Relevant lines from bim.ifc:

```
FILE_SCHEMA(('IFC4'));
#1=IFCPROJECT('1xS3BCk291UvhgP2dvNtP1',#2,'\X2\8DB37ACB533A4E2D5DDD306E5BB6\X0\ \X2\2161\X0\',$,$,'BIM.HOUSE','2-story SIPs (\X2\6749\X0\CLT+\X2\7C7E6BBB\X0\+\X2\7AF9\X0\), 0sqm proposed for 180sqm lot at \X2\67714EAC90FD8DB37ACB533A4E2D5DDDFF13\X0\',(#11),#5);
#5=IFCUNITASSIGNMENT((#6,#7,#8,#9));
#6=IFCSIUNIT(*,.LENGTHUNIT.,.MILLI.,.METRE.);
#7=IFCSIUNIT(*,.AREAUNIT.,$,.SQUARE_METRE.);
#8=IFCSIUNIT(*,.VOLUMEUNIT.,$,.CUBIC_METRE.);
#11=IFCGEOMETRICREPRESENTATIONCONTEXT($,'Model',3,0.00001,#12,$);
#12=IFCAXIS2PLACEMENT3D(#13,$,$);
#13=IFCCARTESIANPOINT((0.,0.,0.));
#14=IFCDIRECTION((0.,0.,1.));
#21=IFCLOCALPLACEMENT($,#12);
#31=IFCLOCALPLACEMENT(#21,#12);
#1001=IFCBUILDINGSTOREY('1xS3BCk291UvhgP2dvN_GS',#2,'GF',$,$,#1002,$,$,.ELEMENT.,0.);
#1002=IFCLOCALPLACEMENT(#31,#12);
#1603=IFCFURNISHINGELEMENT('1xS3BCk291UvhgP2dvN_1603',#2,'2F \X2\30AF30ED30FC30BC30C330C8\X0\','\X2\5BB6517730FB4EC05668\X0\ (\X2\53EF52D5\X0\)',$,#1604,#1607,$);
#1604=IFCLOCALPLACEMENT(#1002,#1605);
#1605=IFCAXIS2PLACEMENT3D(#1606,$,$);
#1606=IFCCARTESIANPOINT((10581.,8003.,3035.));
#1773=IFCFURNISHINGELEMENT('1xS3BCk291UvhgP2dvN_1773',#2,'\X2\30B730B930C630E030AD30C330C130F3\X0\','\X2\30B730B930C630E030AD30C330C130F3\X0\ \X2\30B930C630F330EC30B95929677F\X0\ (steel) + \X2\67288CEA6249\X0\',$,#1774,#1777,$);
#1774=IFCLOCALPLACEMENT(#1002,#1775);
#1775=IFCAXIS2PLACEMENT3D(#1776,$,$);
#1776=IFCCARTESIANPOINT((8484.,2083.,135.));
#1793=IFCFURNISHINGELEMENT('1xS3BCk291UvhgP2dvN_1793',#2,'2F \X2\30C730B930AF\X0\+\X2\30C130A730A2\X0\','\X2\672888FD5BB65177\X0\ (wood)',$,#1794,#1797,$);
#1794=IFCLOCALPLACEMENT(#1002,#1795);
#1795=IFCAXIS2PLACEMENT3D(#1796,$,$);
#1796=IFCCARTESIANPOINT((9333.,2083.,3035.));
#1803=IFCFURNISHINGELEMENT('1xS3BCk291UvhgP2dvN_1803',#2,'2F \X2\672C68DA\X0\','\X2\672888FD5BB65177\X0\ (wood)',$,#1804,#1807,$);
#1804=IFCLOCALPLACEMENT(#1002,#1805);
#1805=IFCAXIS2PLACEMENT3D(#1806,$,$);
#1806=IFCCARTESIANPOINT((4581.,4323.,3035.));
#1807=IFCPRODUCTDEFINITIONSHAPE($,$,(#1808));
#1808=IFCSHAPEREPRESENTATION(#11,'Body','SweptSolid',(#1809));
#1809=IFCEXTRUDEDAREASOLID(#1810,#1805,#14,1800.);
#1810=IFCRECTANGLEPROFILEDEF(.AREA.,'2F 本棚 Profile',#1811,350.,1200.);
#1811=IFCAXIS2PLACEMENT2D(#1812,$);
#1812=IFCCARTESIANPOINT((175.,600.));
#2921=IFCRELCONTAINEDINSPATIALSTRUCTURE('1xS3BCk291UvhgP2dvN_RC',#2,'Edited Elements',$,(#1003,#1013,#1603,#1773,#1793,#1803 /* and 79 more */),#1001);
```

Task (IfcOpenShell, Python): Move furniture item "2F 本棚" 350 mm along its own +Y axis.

```python
import ifcopenshell
import ifcopenshell.api.geometry
import ifcopenshell.util.placement

model = ifcopenshell.open("bim.ifc")

item = model.by_id(1803)
matrix = ifcopenshell.util.placement.get_local_placement(item.ObjectPlacement)
matrix[:3, 3] += matrix[:3, 1] * 350.0
ifcopenshell.api.geometry.edit_object_placement(model, product=item, matrix=matrix, is_si=False)

print(ifcopenshell.util.placement.get_local_placement(item.ObjectPlacement).round(3) + 0.0)

model.write("bim_v2.ifc")
```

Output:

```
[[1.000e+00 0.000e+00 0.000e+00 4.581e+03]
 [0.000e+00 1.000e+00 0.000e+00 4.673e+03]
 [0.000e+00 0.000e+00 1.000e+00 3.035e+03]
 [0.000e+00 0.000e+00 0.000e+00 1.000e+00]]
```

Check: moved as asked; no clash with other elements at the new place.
